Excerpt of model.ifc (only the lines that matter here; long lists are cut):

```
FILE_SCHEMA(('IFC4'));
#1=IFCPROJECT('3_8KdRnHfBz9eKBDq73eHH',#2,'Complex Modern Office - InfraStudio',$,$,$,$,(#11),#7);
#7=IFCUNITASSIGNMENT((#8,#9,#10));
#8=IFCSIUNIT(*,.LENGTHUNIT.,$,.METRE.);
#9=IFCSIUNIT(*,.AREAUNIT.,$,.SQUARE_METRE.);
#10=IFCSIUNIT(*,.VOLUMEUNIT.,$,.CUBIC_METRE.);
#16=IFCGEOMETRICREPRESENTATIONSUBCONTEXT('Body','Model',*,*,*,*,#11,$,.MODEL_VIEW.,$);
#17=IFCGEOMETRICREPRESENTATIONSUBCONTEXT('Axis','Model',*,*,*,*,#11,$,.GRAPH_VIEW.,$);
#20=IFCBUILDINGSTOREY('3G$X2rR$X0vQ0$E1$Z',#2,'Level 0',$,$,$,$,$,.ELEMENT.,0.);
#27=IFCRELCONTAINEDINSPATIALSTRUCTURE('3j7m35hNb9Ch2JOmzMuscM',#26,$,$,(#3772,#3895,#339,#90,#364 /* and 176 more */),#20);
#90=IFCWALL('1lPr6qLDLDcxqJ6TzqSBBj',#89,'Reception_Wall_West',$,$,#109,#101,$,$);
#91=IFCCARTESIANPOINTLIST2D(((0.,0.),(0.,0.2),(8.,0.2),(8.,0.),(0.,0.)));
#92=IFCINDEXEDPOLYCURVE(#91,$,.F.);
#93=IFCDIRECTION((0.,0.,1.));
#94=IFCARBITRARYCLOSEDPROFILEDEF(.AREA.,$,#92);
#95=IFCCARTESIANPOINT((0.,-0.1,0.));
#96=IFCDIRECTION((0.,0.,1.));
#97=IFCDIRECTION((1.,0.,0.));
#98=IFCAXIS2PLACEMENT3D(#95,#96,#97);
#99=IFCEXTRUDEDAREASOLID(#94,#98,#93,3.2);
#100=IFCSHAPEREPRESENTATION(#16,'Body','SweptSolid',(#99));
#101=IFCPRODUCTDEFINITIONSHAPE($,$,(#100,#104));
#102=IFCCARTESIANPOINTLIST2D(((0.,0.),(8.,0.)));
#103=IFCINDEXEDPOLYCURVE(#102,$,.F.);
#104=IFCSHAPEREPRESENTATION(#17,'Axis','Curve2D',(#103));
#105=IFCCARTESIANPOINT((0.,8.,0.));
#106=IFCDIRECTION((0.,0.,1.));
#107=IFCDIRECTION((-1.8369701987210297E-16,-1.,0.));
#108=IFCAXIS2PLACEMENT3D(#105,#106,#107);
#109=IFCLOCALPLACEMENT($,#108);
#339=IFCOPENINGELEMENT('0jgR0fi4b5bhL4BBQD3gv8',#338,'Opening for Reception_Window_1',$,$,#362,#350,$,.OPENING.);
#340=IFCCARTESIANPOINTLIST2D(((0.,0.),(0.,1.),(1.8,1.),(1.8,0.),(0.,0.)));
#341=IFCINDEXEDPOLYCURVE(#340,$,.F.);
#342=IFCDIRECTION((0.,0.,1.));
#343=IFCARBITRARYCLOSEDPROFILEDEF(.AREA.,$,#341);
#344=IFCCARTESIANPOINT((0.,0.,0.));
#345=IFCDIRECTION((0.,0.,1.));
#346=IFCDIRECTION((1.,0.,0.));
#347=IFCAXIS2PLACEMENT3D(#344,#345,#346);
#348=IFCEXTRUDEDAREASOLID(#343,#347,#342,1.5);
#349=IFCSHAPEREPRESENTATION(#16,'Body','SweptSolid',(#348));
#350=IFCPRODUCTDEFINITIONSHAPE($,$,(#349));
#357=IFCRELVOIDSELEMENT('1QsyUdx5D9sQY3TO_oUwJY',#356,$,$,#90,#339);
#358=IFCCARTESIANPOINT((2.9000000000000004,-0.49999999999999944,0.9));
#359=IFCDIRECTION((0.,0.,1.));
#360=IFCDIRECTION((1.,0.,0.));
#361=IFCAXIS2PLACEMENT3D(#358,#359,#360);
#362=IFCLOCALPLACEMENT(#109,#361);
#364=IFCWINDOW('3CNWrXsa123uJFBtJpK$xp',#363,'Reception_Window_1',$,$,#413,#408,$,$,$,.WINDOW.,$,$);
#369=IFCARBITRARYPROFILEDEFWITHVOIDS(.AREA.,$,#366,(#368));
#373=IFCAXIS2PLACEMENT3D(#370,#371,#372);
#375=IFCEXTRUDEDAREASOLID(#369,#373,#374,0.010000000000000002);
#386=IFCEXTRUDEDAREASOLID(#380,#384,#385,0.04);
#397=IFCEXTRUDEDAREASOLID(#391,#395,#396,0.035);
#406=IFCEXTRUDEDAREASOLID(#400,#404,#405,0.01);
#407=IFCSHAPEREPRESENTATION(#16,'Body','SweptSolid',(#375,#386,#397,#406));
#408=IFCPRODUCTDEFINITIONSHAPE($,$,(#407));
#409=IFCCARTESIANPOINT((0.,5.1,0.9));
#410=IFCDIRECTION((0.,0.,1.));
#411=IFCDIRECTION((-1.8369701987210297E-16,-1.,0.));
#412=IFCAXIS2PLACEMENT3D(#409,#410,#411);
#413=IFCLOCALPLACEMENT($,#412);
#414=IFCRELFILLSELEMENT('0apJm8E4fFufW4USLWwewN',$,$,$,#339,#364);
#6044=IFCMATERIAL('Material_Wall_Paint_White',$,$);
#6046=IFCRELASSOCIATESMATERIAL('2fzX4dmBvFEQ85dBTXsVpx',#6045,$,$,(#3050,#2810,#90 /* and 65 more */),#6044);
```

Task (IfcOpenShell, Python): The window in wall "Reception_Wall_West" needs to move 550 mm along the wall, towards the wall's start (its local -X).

```python
import ifcopenshell
import ifcopenshell.api.geometry
import ifcopenshell.util.placement

model = ifcopenshell.open("model.ifc")

window = model.by_id(364)
opening = window.FillsVoids[0].RelatingOpeningElement
wall = opening.VoidsElements[0].RelatingBuildingElement

wall_matrix = ifcopenshell.util.placement.get_local_placement(wall.ObjectPlacement)
shift = wall_matrix[:3, 0] * -0.55
before = ifcopenshell.util.placement.get_local_placement(window.ObjectPlacement)[:3, 3].copy()

# The window is not placed relative to its opening, so move both.
for product in (opening, window):
    matrix = ifcopenshell.util.placement.get_local_placement(product.ObjectPlacement)
    matrix[:3, 3] += shift
    ifcopenshell.api.geometry.edit_object_placement(model, product=product, matrix=matrix, is_si=False)

after = ifcopenshell.util.placement.get_local_placement(window.ObjectPlacement)[:3, 3]
print("window moved by", (after - before).round(3) + 0.0)

model.write("model_rev.ifc")
```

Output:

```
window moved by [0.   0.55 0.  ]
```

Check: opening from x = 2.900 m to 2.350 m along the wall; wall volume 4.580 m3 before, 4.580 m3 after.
